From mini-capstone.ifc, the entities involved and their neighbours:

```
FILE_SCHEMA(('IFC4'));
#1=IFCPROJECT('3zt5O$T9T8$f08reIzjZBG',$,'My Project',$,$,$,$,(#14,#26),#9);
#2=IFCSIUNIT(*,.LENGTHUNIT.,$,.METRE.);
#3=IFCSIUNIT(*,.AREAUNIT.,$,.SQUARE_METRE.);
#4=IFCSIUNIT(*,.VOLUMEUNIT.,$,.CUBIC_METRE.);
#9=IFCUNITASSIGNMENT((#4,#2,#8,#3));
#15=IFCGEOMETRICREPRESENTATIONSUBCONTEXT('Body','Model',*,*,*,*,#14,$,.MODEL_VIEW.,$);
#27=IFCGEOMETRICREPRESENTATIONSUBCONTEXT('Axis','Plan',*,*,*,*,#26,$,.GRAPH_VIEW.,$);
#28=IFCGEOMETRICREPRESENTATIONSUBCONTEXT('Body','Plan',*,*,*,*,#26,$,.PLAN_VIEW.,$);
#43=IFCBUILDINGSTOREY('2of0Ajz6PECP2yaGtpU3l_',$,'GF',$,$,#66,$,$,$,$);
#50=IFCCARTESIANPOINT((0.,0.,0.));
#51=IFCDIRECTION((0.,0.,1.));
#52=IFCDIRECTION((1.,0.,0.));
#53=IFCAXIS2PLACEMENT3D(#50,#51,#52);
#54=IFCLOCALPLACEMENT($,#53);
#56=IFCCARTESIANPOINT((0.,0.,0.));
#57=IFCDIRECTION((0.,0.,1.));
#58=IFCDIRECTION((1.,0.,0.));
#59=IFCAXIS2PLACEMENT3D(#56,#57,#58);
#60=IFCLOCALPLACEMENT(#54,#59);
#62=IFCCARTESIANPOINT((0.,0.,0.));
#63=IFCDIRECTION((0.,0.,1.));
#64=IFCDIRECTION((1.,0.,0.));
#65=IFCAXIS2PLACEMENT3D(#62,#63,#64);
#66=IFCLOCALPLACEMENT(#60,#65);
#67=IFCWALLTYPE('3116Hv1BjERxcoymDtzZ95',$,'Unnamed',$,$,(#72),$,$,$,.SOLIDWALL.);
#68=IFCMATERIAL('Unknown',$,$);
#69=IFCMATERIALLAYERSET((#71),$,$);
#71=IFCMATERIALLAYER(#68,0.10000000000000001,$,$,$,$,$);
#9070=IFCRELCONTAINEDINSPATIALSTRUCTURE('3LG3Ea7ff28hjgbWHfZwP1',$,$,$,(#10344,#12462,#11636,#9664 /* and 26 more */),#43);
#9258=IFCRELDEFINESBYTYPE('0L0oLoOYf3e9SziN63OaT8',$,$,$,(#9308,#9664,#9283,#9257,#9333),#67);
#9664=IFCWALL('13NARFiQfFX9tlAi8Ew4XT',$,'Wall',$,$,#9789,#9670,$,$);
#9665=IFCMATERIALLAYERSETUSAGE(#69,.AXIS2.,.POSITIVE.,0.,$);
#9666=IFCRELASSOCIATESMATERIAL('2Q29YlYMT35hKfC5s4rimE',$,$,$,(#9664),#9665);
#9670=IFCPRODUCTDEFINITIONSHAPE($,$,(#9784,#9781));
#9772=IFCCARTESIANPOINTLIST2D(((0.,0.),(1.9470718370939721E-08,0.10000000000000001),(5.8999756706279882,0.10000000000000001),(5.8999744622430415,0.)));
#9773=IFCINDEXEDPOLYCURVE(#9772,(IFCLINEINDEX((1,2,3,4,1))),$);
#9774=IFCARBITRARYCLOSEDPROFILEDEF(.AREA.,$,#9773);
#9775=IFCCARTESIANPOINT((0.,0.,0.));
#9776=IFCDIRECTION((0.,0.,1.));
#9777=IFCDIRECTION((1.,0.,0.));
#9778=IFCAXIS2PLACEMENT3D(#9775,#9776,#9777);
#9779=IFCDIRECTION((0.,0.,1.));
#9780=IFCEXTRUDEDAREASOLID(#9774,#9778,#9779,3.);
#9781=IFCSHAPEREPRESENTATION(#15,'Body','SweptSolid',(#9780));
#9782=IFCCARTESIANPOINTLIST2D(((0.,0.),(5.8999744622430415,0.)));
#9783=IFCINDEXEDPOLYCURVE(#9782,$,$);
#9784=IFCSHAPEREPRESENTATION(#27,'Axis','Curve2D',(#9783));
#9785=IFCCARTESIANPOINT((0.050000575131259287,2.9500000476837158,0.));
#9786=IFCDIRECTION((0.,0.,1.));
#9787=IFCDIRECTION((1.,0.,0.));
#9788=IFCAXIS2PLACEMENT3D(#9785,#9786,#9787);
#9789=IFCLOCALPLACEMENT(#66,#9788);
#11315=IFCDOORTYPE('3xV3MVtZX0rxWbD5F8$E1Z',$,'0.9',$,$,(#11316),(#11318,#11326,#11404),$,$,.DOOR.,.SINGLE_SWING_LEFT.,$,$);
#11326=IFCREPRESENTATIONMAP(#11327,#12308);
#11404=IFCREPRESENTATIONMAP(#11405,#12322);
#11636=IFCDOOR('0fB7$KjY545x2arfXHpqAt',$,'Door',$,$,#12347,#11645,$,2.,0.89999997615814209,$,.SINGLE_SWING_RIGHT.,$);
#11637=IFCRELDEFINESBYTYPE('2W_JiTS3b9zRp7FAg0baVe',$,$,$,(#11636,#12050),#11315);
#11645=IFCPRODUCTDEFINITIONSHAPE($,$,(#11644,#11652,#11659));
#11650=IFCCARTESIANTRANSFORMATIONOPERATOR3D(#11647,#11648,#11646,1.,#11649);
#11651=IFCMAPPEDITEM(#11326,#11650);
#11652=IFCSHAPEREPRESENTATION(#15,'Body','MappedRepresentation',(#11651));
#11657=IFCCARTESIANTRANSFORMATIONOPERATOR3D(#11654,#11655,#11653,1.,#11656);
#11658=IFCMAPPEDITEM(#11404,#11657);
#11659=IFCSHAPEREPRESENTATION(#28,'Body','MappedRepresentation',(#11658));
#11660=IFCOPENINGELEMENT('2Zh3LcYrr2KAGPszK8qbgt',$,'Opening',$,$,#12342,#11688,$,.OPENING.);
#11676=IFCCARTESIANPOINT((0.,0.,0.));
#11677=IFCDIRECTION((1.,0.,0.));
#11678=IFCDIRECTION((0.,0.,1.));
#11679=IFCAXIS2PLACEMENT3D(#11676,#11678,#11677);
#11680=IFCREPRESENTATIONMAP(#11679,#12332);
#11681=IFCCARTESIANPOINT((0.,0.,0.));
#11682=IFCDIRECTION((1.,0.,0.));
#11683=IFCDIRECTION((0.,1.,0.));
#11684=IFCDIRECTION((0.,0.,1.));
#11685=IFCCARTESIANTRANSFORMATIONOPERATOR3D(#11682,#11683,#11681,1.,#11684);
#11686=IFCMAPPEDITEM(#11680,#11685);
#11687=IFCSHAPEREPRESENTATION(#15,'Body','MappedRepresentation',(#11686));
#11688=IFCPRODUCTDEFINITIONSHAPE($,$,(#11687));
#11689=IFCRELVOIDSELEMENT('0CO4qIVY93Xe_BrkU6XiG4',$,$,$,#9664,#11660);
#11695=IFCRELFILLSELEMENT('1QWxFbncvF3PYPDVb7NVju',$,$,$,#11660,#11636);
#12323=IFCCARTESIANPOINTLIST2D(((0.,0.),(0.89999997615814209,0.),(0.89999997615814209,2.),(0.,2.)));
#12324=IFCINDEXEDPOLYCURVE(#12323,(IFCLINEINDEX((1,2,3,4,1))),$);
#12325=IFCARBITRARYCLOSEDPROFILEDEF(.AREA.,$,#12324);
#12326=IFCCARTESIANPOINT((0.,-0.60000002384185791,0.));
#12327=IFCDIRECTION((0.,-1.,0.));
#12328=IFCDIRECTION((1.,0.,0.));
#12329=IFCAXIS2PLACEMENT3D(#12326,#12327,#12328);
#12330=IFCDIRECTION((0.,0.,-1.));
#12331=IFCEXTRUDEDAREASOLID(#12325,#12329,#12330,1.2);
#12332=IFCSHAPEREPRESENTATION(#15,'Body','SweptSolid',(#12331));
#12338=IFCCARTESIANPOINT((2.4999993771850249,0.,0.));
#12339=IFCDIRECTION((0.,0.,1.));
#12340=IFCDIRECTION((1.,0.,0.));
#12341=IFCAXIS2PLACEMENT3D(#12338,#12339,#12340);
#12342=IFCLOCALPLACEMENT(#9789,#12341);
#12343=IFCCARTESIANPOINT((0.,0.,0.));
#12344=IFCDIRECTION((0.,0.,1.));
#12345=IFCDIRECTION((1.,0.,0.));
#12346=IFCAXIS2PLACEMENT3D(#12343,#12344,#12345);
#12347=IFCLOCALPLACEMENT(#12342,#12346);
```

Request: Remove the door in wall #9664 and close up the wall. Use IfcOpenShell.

```python
import ifcopenshell
import ifcopenshell.api.feature
import ifcopenshell.api.root
import ifcopenshell.geom
import ifcopenshell.util.shape

model = ifcopenshell.open("mini-capstone.ifc")
settings = ifcopenshell.geom.settings()


def volume(element):
    """Net volume in cubic metres, openings subtracted."""
    shape = ifcopenshell.geom.create_shape(settings, element)
    return ifcopenshell.util.shape.get_volume(shape.geometry)


door = model.by_guid("0fB7$KjY545x2arfXHpqAt")
opening = door.FillsVoids[0].RelatingOpeningElement
wall = opening.VoidsElements[0].RelatingBuildingElement
before = volume(wall)

ifcopenshell.api.root.remove_product(model, product=door)
ifcopenshell.api.feature.remove_feature(model, feature=opening)

after = volume(wall)

print(f"wall volume {before:.3f} -> {after:.3f} m3")

model.write("mini-capstone-out.ifc")
```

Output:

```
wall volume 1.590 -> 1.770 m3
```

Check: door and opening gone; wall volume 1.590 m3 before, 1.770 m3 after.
